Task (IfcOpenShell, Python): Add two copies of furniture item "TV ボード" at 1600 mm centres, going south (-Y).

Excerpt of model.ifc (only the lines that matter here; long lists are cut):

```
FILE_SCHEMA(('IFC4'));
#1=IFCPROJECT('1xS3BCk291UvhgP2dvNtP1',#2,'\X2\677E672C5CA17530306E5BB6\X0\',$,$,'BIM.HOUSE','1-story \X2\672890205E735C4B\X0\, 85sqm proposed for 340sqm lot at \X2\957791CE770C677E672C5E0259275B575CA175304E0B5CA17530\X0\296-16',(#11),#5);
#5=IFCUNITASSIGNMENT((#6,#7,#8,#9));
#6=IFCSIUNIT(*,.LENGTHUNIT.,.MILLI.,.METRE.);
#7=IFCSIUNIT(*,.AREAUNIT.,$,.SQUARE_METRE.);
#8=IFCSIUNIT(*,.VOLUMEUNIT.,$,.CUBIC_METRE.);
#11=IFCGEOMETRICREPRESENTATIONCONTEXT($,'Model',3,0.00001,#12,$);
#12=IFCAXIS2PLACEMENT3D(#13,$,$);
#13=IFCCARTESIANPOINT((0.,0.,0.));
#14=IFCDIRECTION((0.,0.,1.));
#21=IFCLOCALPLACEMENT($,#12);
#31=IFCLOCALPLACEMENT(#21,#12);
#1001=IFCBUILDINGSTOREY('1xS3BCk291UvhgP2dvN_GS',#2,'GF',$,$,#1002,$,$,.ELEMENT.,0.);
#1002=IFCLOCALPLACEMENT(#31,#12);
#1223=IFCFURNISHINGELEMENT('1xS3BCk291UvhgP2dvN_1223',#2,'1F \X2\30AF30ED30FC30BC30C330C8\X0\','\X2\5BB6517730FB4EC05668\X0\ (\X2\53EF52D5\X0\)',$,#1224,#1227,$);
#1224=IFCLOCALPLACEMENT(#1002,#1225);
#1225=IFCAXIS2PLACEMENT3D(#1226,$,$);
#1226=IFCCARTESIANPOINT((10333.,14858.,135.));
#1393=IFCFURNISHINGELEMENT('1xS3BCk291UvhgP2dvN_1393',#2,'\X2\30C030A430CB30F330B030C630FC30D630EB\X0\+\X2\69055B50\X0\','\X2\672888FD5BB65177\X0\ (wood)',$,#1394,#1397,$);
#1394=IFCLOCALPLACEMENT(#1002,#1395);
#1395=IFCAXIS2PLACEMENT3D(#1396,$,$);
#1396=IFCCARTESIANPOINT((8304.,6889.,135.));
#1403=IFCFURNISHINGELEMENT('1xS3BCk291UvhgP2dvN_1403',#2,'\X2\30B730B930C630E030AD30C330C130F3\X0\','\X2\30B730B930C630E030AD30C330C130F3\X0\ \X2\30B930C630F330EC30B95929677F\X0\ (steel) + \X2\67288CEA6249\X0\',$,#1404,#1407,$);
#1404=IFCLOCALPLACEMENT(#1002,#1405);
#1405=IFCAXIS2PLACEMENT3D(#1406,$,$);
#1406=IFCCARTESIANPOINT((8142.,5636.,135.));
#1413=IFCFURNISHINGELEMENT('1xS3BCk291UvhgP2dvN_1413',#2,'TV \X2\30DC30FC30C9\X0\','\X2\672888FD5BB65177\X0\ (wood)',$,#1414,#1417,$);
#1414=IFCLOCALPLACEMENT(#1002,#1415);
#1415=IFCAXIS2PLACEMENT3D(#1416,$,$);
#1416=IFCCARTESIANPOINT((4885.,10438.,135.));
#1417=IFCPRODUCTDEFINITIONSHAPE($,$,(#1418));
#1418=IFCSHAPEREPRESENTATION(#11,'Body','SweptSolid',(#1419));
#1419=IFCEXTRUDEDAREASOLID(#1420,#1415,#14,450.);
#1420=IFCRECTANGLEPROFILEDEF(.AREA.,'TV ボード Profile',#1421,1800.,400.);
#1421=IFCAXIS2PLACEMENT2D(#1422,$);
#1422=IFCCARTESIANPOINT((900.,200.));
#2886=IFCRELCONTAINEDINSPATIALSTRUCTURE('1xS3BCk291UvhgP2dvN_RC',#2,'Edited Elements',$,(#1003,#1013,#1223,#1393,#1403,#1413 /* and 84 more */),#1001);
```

```python
import numpy as np
import ifcopenshell
import ifcopenshell.api.geometry
import ifcopenshell.api.root
import ifcopenshell.util.element
import ifcopenshell.util.placement
import ifcopenshell.util.unit

model = ifcopenshell.open("model.ifc")
unit_scale = ifcopenshell.util.unit.calculate_unit_scale(model)


def reuse_history(source, copy):
    """copy_class also copies each property set's owner history, people and application; keep the originals."""
    for rel in copy.IsDefinedBy:
        if rel.is_a("IfcRelDefinesByProperties") and (history := rel.RelatingPropertyDefinition.OwnerHistory):
            rel.RelatingPropertyDefinition.OwnerHistory = source.OwnerHistory
            ifcopenshell.util.element.remove_deep2(model, history)


source = model.by_guid("1xS3BCk291UvhgP2dvN_1413")
base = ifcopenshell.util.placement.get_local_placement(source.ObjectPlacement)
step = np.array([0.0, -1.0, 0.0]) * 1.6 / unit_scale

for i in range(1, 3):
    copy = ifcopenshell.api.root.copy_class(model, product=source)
    copy.Representation = ifcopenshell.util.element.copy_deep(
        model, source.Representation, exclude=["IfcGeometricRepresentationContext", "IfcRepresentationMap"]
    )
    reuse_history(source, copy)
    matrix = base.copy()
    matrix[:3, 3] += i * step
    print("added at", matrix[:3, 3].round(3) + 0.0)
    ifcopenshell.api.geometry.edit_object_placement(model, product=copy, matrix=matrix, is_si=False)

model.write("model_v2.ifc")
```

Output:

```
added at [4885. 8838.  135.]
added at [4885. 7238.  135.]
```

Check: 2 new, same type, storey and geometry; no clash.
